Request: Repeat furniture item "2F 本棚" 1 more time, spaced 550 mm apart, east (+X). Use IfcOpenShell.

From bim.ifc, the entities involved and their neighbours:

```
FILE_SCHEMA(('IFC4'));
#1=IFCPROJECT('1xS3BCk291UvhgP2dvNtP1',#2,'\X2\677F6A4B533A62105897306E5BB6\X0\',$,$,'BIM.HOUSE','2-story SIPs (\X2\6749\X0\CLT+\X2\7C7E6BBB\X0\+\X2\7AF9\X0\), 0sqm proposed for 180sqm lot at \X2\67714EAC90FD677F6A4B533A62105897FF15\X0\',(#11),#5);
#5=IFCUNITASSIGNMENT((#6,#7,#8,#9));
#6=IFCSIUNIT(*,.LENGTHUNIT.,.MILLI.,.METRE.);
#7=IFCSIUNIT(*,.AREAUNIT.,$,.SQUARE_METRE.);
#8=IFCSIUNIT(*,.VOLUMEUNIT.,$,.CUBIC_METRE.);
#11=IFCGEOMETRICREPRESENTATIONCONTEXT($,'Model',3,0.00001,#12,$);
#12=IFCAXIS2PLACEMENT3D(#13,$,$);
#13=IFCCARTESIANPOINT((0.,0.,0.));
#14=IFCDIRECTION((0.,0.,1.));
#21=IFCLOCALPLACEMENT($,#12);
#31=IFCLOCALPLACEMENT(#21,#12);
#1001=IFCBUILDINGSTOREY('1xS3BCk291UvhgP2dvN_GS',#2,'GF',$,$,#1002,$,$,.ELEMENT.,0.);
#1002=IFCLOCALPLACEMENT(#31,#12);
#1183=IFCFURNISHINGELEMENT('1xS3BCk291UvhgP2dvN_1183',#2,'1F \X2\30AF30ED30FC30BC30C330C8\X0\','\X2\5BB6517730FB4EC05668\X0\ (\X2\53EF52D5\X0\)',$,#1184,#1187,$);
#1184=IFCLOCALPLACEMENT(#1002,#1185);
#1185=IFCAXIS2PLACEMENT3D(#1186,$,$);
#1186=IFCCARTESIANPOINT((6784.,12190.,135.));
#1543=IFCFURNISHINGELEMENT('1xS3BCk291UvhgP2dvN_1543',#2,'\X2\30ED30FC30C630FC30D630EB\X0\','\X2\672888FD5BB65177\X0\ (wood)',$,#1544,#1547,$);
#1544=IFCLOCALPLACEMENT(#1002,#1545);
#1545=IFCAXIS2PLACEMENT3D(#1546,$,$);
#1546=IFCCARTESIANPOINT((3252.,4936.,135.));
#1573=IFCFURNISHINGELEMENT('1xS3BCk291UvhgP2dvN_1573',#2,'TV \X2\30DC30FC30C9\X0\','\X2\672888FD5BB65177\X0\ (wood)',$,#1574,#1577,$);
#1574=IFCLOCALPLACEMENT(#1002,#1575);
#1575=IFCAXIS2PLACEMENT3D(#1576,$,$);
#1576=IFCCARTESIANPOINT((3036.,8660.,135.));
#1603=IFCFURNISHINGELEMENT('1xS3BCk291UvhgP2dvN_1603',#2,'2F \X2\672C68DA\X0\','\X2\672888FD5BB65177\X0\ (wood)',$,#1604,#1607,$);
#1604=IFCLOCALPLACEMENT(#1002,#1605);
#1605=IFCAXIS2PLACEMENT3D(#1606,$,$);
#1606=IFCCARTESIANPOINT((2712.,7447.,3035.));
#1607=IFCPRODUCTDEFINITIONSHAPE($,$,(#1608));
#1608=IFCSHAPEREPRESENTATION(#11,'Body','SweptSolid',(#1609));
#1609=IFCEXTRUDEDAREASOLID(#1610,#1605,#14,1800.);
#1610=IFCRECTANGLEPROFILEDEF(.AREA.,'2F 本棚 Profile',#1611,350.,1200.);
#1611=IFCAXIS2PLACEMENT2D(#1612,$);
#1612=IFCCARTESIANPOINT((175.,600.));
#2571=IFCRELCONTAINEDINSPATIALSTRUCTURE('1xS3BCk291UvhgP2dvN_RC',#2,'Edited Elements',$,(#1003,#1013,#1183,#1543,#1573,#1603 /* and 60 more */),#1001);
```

```python
import numpy as np
import ifcopenshell
import ifcopenshell.api.geometry
import ifcopenshell.api.root
import ifcopenshell.util.element
import ifcopenshell.util.placement

model = ifcopenshell.open("bim.ifc")


def reuse_history(source, copy):
    """copy_class also copies each property set's owner history, people and application; keep the originals."""
    for rel in copy.IsDefinedBy:
        if rel.is_a("IfcRelDefinesByProperties") and (history := rel.RelatingPropertyDefinition.OwnerHistory):
            rel.RelatingPropertyDefinition.OwnerHistory = source.OwnerHistory
            ifcopenshell.util.element.remove_deep2(model, history)


source = model.by_guid("1xS3BCk291UvhgP2dvN_1603")
base = ifcopenshell.util.placement.get_local_placement(source.ObjectPlacement)
step = np.array([1.0, 0.0, 0.0]) * 550.0

for i in range(1, 2):
    copy = ifcopenshell.api.root.copy_class(model, product=source)
    copy.Representation = ifcopenshell.util.element.copy_deep(
        model, source.Representation, exclude=["IfcGeometricRepresentationContext", "IfcRepresentationMap"]
    )
    reuse_history(source, copy)
    matrix = base.copy()
    matrix[:3, 3] += i * step
    print("added at", matrix[:3, 3].round(3) + 0.0)
    ifcopenshell.api.geometry.edit_object_placement(model, product=copy, matrix=matrix, is_si=False)

model.write("bim_updated.ifc")
```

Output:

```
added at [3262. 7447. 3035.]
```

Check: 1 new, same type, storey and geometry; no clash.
